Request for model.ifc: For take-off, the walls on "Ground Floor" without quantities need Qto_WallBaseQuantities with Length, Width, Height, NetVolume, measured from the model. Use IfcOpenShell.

First a look at what the model holds.

```python
import ifcopenshell
import ifcopenshell.util.element
import ifcopenshell.util.unit

model = ifcopenshell.open("model.ifc")
print(model.schema)
for unit_type in ("LENGTHUNIT", "AREAUNIT", "VOLUMEUNIT"):
    print(unit_type, ifcopenshell.util.unit.calculate_unit_scale(model, unit_type))
storey = next(s for s in model.by_type("IfcBuildingStorey") if s.Name == "Ground Floor")
walls = [e for e in ifcopenshell.util.element.get_decomposition(storey) if e.is_a("IfcWall")]
for e in sorted(walls, key=lambda e: e.id()):
    print(e.id(), e.is_a(), e.Name, list(ifcopenshell.util.element.get_psets(e, qtos_only=True)), sep=" | ")
```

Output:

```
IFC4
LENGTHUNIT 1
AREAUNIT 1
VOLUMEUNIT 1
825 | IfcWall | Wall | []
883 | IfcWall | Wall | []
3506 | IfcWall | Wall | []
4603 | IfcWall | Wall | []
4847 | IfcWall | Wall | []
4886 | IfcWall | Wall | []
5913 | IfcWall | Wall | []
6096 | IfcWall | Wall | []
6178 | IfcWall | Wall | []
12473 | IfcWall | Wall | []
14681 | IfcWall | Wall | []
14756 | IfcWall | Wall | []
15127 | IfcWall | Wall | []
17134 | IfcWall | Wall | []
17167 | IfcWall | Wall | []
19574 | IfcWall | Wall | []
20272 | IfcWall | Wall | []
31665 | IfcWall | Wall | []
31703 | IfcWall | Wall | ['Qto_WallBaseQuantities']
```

```python
import ifcopenshell
import ifcopenshell.api.pset
import ifcopenshell.geom
import ifcopenshell.util.element
import ifcopenshell.util.shape
import ifcopenshell.util.unit

model = ifcopenshell.open("model.ifc")
unit_scale = ifcopenshell.util.unit.calculate_unit_scale(model)
volume_scale = ifcopenshell.util.unit.calculate_unit_scale(model, "VOLUMEUNIT")
settings = ifcopenshell.geom.settings()

storey = next(s for s in model.by_type("IfcBuildingStorey") if s.Name == "Ground Floor")
walls = [e for e in ifcopenshell.util.element.get_decomposition(storey) if e.is_a("IfcWall")]

for e in sorted(walls, key=lambda e: e.id()):
    if ifcopenshell.util.element.get_psets(e, qtos_only=True, should_inherit=False):
        continue
    # Geometry comes back in metres, in the element's own axes.
    shape = ifcopenshell.geom.create_shape(settings, e)
    values = {
        "Length": ifcopenshell.util.shape.get_x(shape.geometry) / unit_scale,
        "Width": ifcopenshell.util.shape.get_y(shape.geometry) / unit_scale,
        "Height": ifcopenshell.util.shape.get_z(shape.geometry) / unit_scale,
        "NetVolume": ifcopenshell.util.shape.get_volume(shape.geometry) / volume_scale,
    }
    qto = ifcopenshell.api.pset.add_qto(model, product=e, name="Qto_WallBaseQuantities")
    ifcopenshell.api.pset.edit_qto(model, qto=qto, properties=values)
    print(e.id(), {k: round(v, 3) for k, v in values.items()})

model.write("model_updated.ifc")
```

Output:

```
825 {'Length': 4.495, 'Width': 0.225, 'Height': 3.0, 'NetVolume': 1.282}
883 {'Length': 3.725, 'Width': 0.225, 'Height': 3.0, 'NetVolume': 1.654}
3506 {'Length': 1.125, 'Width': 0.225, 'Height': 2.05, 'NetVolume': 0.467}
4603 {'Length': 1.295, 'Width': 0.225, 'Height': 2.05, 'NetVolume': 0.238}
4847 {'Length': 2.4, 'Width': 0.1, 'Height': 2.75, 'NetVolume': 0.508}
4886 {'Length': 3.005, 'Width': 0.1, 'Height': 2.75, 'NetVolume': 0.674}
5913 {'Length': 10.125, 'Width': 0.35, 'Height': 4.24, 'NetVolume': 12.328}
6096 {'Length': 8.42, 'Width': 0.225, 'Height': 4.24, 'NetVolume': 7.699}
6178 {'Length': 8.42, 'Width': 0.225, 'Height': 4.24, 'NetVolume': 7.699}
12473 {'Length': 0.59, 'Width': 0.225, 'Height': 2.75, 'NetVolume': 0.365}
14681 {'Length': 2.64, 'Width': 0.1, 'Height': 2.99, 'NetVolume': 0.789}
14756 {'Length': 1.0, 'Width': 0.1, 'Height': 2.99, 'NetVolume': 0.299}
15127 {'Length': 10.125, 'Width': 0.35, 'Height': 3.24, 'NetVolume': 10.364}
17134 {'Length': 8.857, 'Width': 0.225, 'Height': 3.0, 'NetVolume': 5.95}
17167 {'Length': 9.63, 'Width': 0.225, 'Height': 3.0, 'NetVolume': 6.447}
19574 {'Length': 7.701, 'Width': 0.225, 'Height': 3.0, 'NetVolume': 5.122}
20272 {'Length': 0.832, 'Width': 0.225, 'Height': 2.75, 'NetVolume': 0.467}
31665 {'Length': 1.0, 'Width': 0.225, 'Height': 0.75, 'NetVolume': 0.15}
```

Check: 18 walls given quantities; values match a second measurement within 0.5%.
